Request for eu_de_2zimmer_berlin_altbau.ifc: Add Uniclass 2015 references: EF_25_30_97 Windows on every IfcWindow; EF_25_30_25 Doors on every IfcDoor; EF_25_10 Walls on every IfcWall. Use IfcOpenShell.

First a look at what the model holds.

```python
import ifcopenshell

model = ifcopenshell.open("eu_de_2zimmer_berlin_altbau.ifc")
print(model.schema)
print("classifications:", [c.Name for c in model.by_type("IfcClassification")])
for ifc_class in ("IfcDoor", "IfcRoof", "IfcStair", "IfcWall", "IfcWindow"):
    print(ifc_class, len(model.by_type(ifc_class)))
```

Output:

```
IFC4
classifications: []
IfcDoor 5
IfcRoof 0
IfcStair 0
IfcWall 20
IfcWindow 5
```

```python
import ifcopenshell
import ifcopenshell.api.classification

model = ifcopenshell.open("eu_de_2zimmer_berlin_altbau.ifc")

system = ifcopenshell.api.classification.add_classification(model, classification="Uniclass 2015")

codes = {
    "IfcWindow": ("EF_25_30_97", "Windows"),
    "IfcDoor": ("EF_25_30_25", "Doors"),
    "IfcWall": ("EF_25_10", "Walls"),
}
for ifc_class, (code, name) in codes.items():
    products = model.by_type(ifc_class)
    ifcopenshell.api.classification.add_reference(
        model, products=products, classification=system, identification=code, name=name
    )
    print(code, len(products))

model.write("eu_de_2zimmer_berlin_altbau_rev.ifc")
```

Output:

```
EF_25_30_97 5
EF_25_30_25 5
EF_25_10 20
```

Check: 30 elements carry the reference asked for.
